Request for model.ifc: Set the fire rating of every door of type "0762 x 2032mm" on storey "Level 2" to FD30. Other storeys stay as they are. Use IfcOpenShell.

First a look at what the model holds.

```python
import ifcopenshell
import ifcopenshell.util.element

model = ifcopenshell.open("model.ifc")
print(model.schema)
storey = next(s for s in model.by_type("IfcBuildingStorey") if s.Name == "Level 2")
doors = [e for e in ifcopenshell.util.element.get_decomposition(storey) if e.is_a("IfcDoor")]
seen = {}
for e in doors:
    element_type = ifcopenshell.util.element.get_type(e)
    key = (element_type.Name if element_type != e and element_type else None, ifcopenshell.util.element.get_pset(e, "Pset_DoorCommon", "FireRating"))
    seen[key] = seen.get(key, 0) + 1
for (name, value), count in sorted(seen.items(), key=str):
    print(count, "x", name, "|", value)
```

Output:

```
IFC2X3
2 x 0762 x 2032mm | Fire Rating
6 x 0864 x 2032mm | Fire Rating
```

```python
import ifcopenshell
import ifcopenshell.api.pset
import ifcopenshell.util.element

model = ifcopenshell.open("model.ifc")

storey = next(s for s in model.by_type("IfcBuildingStorey") if s.Name == "Level 2")
doors = [e for e in ifcopenshell.util.element.get_decomposition(storey) if e.is_a("IfcDoor")]

count = 0
for e in doors:
    element_type = ifcopenshell.util.element.get_type(e)
    if element_type in (None, e) or element_type.Name != "0762 x 2032mm":
        continue
    # add_pset returns the element's existing set when there is one.
    pset = ifcopenshell.api.pset.add_pset(model, product=e, name="Pset_DoorCommon")
    ifcopenshell.api.pset.edit_pset(model, pset=pset, properties={"FireRating": "FD30"})
    count += 1

print(count, "doors updated")

model.write("model_edited.ifc")
```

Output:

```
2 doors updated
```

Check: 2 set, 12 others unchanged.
